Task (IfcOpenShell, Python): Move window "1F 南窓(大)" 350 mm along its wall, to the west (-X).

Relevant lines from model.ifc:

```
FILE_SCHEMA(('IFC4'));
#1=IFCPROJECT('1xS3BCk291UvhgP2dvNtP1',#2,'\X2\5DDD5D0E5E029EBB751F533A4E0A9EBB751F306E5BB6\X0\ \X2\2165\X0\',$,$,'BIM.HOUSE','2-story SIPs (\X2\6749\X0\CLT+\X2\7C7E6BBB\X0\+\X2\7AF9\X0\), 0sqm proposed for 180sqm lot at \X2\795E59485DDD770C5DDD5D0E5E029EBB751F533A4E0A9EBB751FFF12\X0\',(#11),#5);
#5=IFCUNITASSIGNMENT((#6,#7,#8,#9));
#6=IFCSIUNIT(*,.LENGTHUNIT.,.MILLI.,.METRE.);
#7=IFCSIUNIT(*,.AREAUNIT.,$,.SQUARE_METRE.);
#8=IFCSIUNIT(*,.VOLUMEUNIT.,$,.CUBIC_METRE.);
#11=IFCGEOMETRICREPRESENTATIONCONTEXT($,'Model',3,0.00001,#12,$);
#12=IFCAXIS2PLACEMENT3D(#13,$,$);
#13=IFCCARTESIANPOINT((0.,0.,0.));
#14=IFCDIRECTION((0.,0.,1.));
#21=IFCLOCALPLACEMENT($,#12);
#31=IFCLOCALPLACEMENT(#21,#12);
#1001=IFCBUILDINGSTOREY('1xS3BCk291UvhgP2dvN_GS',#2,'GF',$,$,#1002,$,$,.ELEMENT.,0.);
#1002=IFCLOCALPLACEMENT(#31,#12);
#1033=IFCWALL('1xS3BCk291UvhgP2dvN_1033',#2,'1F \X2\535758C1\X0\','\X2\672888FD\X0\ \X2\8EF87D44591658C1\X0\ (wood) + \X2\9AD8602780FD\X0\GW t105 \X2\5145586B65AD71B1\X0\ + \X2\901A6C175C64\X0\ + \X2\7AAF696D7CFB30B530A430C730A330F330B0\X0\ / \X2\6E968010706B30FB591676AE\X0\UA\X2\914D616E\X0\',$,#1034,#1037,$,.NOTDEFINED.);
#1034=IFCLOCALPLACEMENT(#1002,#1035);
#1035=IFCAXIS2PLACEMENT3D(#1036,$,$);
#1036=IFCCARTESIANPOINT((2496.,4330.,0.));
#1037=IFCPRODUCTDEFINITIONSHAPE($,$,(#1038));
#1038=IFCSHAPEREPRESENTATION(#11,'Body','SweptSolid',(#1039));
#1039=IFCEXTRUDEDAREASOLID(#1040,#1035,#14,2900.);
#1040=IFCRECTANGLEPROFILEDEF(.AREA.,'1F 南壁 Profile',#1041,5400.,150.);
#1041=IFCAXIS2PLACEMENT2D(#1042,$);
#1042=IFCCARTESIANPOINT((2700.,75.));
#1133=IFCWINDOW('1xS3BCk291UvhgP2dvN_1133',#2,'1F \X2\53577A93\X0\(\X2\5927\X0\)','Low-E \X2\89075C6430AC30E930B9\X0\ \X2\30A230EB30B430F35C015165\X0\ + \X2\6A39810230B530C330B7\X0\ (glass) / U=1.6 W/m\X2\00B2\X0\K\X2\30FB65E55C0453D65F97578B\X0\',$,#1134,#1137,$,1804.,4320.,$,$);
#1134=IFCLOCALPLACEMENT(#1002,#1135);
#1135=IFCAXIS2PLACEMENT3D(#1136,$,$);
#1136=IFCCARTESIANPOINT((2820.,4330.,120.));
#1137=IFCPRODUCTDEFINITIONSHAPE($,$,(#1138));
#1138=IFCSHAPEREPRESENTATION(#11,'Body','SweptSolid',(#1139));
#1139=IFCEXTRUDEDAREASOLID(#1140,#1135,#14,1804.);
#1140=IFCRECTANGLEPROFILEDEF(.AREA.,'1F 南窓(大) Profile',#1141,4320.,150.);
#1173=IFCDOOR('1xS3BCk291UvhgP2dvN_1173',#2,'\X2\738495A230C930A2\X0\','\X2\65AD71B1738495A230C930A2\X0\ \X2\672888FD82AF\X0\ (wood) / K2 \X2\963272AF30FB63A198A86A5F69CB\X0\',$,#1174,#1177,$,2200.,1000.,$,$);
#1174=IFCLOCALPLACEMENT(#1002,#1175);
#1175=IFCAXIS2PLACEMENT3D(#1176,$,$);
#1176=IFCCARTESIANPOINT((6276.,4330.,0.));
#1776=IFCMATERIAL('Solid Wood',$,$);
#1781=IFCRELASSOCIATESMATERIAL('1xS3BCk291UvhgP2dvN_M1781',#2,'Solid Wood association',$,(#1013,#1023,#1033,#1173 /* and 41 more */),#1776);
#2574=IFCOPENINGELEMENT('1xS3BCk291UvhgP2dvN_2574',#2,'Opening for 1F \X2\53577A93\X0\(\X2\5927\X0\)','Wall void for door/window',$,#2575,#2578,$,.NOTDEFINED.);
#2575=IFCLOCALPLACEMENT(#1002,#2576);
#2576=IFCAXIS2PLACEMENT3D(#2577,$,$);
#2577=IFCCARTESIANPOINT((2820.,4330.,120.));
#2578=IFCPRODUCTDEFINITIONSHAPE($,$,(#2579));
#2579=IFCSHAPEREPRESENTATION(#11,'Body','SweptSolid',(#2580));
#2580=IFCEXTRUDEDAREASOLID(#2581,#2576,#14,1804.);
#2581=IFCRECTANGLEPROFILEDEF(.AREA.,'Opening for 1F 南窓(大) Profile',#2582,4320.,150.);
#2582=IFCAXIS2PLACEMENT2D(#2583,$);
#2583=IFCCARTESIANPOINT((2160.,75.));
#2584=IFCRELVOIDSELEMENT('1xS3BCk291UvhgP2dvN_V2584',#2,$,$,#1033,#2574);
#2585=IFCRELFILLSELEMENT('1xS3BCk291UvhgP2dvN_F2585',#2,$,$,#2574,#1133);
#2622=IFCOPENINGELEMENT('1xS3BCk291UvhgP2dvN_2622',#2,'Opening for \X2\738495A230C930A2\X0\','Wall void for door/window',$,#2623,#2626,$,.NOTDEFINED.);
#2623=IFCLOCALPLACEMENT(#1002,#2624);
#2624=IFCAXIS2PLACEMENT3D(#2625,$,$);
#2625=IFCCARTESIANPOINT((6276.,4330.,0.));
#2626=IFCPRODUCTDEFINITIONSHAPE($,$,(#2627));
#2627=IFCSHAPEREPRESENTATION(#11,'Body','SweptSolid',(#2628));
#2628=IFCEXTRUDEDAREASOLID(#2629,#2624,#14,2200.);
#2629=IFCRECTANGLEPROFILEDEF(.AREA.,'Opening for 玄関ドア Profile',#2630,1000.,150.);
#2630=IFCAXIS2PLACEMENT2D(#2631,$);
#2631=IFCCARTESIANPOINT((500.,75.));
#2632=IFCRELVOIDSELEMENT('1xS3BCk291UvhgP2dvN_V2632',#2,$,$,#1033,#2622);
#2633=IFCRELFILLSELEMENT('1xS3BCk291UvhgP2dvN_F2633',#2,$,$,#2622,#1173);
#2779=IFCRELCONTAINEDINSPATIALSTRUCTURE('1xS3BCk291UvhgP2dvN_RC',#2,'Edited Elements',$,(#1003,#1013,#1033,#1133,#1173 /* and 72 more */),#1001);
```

```python
import ifcopenshell
import ifcopenshell.api.geometry
import ifcopenshell.util.placement
import ifcopenshell.util.unit

model = ifcopenshell.open("model.ifc")
unit_scale = ifcopenshell.util.unit.calculate_unit_scale(model)

window = model.by_guid("1xS3BCk291UvhgP2dvN_1133")
opening = window.FillsVoids[0].RelatingOpeningElement
wall = opening.VoidsElements[0].RelatingBuildingElement

wall_matrix = ifcopenshell.util.placement.get_local_placement(wall.ObjectPlacement)
shift = wall_matrix[:3, 0] * -0.35 / unit_scale
before = ifcopenshell.util.placement.get_local_placement(window.ObjectPlacement)[:3, 3].copy()

# The window is not placed relative to its opening, so move both.
for product in (opening, window):
    matrix = ifcopenshell.util.placement.get_local_placement(product.ObjectPlacement)
    matrix[:3, 3] += shift
    ifcopenshell.api.geometry.edit_object_placement(model, product=product, matrix=matrix, is_si=False)

after = ifcopenshell.util.placement.get_local_placement(window.ObjectPlacement)[:3, 3]
print("window moved by", (after - before).round(3) + 0.0)

model.write("model-out.ifc")
```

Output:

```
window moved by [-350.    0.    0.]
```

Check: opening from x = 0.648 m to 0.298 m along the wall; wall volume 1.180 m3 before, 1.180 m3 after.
